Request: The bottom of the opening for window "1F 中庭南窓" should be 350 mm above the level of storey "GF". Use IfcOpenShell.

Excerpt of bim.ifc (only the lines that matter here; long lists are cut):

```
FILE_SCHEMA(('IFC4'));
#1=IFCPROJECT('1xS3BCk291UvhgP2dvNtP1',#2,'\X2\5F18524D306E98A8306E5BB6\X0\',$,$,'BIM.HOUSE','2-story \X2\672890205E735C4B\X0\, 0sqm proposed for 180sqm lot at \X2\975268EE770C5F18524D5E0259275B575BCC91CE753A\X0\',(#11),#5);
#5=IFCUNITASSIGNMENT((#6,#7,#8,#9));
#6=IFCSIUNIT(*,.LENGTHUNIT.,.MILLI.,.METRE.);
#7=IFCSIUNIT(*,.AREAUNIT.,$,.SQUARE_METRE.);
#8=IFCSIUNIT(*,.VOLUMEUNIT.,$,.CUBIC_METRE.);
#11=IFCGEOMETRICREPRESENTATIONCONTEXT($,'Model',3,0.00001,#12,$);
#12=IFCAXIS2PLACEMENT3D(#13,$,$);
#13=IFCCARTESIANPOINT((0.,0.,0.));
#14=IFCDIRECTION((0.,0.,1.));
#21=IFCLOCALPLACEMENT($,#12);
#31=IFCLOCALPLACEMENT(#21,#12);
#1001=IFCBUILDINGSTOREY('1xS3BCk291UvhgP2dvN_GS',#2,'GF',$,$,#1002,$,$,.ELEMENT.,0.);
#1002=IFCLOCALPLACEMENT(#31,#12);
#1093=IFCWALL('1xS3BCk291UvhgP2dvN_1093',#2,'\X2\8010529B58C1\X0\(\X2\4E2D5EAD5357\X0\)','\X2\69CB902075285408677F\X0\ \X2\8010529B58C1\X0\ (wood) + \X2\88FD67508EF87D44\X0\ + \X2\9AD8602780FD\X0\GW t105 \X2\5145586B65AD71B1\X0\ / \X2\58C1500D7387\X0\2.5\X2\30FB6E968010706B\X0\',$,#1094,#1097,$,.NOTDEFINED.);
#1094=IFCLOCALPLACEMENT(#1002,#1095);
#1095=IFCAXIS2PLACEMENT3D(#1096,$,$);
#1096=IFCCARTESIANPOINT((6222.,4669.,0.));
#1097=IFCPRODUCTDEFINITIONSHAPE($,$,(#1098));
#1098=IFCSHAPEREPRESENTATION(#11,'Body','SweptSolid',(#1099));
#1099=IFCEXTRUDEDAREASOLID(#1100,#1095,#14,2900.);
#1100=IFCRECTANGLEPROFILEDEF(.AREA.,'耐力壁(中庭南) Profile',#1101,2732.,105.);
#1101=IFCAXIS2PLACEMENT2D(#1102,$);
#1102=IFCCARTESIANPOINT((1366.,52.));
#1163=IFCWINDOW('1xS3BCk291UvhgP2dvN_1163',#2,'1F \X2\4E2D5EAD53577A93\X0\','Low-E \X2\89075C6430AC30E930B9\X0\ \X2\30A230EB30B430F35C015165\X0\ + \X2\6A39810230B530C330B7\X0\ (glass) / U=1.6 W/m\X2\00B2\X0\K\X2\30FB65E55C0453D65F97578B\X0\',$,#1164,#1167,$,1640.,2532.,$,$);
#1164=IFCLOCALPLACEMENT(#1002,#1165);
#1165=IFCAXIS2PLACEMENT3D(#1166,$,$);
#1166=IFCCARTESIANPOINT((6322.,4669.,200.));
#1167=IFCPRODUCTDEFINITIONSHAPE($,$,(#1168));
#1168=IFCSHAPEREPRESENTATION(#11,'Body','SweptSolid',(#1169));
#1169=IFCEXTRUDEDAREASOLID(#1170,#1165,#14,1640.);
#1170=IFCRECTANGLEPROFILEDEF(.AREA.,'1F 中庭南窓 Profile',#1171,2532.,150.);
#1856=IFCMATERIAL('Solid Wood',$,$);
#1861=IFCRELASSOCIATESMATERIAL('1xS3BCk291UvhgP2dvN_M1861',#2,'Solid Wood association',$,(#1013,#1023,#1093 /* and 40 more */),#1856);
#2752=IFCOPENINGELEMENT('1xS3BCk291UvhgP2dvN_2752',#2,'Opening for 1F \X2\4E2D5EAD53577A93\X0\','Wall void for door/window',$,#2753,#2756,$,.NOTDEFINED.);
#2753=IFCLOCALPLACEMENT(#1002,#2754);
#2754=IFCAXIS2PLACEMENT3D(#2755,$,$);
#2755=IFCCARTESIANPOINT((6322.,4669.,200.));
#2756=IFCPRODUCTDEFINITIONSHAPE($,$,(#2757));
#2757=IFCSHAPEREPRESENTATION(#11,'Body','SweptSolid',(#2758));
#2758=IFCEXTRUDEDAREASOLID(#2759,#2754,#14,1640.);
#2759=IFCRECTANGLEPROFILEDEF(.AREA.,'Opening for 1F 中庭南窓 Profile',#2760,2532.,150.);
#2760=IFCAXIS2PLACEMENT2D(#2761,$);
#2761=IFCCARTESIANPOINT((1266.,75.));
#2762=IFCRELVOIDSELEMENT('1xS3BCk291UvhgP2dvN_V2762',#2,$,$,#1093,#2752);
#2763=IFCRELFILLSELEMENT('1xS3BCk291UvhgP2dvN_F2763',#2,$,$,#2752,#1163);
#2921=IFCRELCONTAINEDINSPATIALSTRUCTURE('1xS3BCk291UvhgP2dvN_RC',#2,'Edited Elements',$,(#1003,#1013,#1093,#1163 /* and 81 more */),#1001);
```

```python
import numpy as np
import ifcopenshell
import ifcopenshell.api.geometry
import ifcopenshell.geom
import ifcopenshell.util.element
import ifcopenshell.util.placement
import ifcopenshell.util.shape
import ifcopenshell.util.unit

model = ifcopenshell.open("bim.ifc")
unit_scale = ifcopenshell.util.unit.calculate_unit_scale(model)

window = model.by_guid("1xS3BCk291UvhgP2dvN_1163")
opening = window.FillsVoids[0].RelatingOpeningElement
storey = ifcopenshell.util.element.get_container(window, ifc_class="IfcBuildingStorey")
level = ifcopenshell.util.placement.get_local_placement(storey.ObjectPlacement)[2, 3]

# The opening's origin need not be at the sill, so measure its lowest point.
shape = ifcopenshell.geom.create_shape(ifcopenshell.geom.settings(), opening)
bottom = ifcopenshell.util.shape.get_shape_bottom_elevation(shape, shape.geometry) / unit_scale
dz = level + 0.35 / unit_scale - bottom

shift = np.array([0.0, 0.0, dz])
# The window is not placed relative to its opening, so move both.
for product in (opening, window):
    matrix = ifcopenshell.util.placement.get_local_placement(product.ObjectPlacement)
    matrix[:3, 3] += shift
    ifcopenshell.api.geometry.edit_object_placement(model, product=product, matrix=matrix, is_si=False)

print(f"moved by {dz * unit_scale:+.3f} m")

model.write("bim_v2.ifc")
```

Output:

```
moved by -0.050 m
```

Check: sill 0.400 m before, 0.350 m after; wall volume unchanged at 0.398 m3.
